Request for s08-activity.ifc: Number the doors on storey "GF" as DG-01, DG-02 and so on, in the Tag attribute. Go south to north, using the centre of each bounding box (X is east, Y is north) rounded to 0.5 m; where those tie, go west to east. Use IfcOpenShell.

First a look at what the model holds.

```python
import ifcopenshell
import ifcopenshell.util.element
import ifcopenshell.util.placement

model = ifcopenshell.open("s08-activity.ifc")
print(model.schema)
storey = next(s for s in model.by_type("IfcBuildingStorey") if s.Name == "GF")
doors = [e for e in ifcopenshell.util.element.get_decomposition(storey) if e.is_a("IfcDoor")]
for e in sorted(doors, key=lambda e: e.id()):
    origin = ifcopenshell.util.placement.get_local_placement(e.ObjectPlacement)[:3, 3]
    print(e.id(), e.Tag, e.Name, origin.round(2) + 0.0, sep=" | ")
```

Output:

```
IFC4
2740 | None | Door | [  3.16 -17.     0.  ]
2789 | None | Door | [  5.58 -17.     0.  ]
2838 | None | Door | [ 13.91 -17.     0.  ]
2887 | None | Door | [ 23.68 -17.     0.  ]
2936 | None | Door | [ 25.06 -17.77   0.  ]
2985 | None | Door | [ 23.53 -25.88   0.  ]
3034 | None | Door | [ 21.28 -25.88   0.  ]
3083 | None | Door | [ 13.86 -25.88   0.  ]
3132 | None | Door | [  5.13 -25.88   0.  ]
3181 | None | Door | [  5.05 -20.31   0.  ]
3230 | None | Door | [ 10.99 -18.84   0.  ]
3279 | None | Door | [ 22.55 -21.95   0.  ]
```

```python
import ifcopenshell
import ifcopenshell.geom
import ifcopenshell.util.element
import ifcopenshell.util.shape

model = ifcopenshell.open("s08-activity.ifc")
settings = ifcopenshell.geom.settings()
settings.set("use-world-coords", True)


def centre(element):
    shape = ifcopenshell.geom.create_shape(settings, element)
    return ifcopenshell.util.shape.get_bbox_centroid(shape.geometry)


storey = next(s for s in model.by_type("IfcBuildingStorey") if s.Name == "GF")
doors = [e for e in ifcopenshell.util.element.get_decomposition(storey) if e.is_a("IfcDoor")]

# Insertion points can sit at a corner or the storey origin, so sort by the geometry (in metres).
centres = {e: centre(e) for e in doors}
doors.sort(key=lambda e: (round(centres[e][1] / 0.5), centres[e][0]))

for i, e in enumerate(doors, start=1):
    number = f"DG-{i:02d}"
    e.Tag = number
    print(e.id(), number)

model.write("s08-activity_edited.ifc")
```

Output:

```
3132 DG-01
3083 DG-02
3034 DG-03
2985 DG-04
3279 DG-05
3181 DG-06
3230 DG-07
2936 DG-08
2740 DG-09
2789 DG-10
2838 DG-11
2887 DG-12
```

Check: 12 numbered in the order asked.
